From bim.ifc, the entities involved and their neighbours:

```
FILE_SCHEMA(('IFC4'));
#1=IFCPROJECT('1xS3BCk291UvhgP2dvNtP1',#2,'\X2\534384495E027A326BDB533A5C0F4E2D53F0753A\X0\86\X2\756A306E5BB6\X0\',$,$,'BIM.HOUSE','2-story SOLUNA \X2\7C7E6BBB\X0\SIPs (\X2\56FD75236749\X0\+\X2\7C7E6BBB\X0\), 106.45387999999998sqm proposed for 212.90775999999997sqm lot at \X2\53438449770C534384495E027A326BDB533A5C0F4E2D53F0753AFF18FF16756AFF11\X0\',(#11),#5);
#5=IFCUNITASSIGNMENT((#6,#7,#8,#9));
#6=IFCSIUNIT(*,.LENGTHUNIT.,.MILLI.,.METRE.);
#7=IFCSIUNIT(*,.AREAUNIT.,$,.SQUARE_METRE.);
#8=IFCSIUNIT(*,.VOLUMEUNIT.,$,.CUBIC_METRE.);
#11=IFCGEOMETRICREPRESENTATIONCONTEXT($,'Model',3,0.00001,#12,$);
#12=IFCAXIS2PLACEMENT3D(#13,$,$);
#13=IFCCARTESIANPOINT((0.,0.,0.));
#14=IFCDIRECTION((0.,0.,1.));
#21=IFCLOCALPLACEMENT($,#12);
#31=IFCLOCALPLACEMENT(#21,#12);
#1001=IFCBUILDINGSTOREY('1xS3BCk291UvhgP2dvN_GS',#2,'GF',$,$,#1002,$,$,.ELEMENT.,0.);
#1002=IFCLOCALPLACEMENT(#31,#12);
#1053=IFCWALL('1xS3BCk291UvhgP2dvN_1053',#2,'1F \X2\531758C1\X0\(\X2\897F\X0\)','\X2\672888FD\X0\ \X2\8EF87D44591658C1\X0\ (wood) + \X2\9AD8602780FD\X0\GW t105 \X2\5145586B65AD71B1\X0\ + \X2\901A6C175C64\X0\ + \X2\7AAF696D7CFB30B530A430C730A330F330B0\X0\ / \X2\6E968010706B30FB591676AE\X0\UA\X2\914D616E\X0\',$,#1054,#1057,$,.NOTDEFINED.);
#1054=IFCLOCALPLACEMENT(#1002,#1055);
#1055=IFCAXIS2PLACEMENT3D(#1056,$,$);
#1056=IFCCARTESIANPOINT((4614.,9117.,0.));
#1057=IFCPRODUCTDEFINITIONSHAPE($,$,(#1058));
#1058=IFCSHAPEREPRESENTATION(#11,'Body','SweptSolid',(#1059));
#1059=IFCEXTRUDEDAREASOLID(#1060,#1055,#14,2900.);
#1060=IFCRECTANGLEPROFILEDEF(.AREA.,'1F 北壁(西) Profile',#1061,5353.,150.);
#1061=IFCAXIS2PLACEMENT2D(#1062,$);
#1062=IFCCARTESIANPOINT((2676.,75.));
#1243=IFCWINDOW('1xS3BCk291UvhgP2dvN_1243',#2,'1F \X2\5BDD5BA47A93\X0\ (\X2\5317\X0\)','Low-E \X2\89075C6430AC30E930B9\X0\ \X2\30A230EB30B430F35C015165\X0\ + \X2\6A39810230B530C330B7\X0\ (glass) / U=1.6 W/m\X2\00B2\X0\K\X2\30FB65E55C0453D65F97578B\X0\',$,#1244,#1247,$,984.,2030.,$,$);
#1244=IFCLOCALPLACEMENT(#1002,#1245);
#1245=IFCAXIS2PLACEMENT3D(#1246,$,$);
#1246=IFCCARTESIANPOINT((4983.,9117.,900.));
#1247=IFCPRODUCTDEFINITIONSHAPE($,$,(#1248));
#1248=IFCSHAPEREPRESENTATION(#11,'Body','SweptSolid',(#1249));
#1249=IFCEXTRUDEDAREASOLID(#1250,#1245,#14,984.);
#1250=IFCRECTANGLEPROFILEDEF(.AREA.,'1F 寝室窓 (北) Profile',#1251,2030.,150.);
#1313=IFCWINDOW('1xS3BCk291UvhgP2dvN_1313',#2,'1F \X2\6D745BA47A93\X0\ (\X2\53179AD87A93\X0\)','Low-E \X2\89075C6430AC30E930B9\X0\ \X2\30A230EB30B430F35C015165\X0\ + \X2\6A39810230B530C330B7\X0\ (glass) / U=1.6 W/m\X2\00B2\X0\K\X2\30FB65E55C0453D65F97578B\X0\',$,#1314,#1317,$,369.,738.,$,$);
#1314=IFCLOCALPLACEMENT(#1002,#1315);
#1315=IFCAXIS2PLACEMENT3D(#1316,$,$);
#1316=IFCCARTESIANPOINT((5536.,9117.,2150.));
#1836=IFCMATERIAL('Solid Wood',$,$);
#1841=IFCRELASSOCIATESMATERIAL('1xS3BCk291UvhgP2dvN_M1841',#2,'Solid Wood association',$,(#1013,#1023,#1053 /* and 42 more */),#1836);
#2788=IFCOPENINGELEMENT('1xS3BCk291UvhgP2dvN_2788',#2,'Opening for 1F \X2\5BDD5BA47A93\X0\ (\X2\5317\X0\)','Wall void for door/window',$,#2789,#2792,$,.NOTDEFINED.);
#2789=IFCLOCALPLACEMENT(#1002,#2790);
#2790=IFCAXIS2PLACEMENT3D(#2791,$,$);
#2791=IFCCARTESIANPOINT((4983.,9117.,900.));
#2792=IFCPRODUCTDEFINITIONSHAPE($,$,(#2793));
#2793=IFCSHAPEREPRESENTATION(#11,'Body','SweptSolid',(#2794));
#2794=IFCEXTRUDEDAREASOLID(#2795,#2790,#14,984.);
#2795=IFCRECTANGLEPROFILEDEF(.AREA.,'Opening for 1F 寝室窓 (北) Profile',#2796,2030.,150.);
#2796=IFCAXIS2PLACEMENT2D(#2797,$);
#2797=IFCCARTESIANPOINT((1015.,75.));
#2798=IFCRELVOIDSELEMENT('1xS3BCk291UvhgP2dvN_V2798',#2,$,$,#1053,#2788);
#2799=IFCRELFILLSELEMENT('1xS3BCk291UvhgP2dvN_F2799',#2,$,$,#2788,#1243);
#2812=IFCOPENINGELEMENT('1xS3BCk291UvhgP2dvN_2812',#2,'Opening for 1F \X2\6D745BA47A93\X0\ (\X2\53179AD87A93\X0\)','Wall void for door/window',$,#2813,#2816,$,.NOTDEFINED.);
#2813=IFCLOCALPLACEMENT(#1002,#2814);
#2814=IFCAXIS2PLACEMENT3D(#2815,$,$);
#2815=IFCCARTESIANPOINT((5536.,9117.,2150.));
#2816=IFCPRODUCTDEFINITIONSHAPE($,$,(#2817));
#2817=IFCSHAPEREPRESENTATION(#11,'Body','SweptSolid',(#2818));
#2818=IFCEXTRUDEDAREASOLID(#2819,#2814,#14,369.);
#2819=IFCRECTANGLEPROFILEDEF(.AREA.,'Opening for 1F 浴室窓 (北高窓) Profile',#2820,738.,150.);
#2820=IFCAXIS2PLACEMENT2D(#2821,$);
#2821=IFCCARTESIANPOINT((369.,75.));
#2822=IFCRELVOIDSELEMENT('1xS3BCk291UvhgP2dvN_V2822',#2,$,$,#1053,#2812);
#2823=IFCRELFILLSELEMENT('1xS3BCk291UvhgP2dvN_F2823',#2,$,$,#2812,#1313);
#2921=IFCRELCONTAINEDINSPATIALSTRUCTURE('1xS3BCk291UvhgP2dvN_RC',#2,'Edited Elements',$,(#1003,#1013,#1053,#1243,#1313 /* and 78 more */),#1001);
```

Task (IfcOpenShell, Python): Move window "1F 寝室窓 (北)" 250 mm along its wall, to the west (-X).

```python
import ifcopenshell
import ifcopenshell.api.geometry
import ifcopenshell.util.placement
import ifcopenshell.util.unit

model = ifcopenshell.open("bim.ifc")
unit_scale = ifcopenshell.util.unit.calculate_unit_scale(model)

window = model.by_guid("1xS3BCk291UvhgP2dvN_1243")
opening = window.FillsVoids[0].RelatingOpeningElement
wall = opening.VoidsElements[0].RelatingBuildingElement

wall_matrix = ifcopenshell.util.placement.get_local_placement(wall.ObjectPlacement)
shift = wall_matrix[:3, 0] * -0.25 / unit_scale
before = ifcopenshell.util.placement.get_local_placement(window.ObjectPlacement)[:3, 3].copy()

# The window is not placed relative to its opening, so move both.
for product in (opening, window):
    matrix = ifcopenshell.util.placement.get_local_placement(product.ObjectPlacement)
    matrix[:3, 3] += shift
    ifcopenshell.api.geometry.edit_object_placement(model, product=product, matrix=matrix, is_si=False)

after = ifcopenshell.util.placement.get_local_placement(window.ObjectPlacement)[:3, 3]
print("window moved by", (after - before).round(3) + 0.0)

model.write("bim_rev.ifc")
```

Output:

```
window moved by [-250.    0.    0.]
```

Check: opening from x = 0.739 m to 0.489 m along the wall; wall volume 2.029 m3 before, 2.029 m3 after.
